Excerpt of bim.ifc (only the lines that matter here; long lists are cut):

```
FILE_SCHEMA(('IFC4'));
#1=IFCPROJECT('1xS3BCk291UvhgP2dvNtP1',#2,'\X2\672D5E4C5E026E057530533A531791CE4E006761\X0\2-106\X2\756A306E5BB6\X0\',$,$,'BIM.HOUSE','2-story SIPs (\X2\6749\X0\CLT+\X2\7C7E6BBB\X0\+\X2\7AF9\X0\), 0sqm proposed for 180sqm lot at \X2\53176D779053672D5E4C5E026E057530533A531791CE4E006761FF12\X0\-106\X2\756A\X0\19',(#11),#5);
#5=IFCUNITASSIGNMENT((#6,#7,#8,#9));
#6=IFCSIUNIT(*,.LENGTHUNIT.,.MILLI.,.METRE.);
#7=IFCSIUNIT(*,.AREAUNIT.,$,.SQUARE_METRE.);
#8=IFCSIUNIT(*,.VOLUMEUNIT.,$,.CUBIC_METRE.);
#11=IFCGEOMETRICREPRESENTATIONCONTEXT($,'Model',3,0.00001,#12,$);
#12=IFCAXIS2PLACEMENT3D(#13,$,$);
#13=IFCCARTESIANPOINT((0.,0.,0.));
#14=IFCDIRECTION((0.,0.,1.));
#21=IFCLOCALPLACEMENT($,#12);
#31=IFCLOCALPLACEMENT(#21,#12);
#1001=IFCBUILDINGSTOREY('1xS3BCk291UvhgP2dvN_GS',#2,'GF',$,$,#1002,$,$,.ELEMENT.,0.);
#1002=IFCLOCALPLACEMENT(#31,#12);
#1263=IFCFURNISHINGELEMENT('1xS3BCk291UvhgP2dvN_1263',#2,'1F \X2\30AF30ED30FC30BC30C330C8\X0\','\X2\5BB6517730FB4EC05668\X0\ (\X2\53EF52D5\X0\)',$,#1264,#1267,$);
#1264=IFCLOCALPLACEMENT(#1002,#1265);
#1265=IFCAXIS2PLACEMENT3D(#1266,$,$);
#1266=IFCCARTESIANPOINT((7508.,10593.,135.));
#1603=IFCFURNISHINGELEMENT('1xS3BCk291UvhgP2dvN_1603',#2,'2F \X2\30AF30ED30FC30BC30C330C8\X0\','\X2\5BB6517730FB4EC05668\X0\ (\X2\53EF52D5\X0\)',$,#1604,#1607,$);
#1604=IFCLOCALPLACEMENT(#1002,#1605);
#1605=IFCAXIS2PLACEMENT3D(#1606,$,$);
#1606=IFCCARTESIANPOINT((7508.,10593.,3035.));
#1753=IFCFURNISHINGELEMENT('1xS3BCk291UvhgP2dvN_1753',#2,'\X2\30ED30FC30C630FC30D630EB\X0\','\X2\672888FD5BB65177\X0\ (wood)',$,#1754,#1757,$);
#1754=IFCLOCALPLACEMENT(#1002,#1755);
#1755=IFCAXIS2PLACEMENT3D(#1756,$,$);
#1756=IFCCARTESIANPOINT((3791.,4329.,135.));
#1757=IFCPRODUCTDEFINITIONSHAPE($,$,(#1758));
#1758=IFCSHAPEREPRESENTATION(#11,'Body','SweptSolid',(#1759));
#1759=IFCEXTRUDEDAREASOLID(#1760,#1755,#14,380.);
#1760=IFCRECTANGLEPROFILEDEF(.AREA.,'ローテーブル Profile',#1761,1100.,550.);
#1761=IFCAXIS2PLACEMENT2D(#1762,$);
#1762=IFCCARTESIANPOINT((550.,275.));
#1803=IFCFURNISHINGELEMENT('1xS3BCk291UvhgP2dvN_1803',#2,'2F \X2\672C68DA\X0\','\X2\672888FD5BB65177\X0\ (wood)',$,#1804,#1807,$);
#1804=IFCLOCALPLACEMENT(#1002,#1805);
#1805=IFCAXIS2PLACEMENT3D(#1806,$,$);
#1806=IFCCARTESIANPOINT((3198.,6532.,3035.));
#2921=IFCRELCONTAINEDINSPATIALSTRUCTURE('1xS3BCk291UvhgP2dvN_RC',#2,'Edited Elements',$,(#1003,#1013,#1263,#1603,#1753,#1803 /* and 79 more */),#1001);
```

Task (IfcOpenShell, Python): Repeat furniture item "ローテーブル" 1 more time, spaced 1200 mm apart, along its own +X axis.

```python
import ifcopenshell
import ifcopenshell.api.geometry
import ifcopenshell.api.root
import ifcopenshell.util.element
import ifcopenshell.util.placement
import ifcopenshell.util.unit

model = ifcopenshell.open("bim.ifc")
unit_scale = ifcopenshell.util.unit.calculate_unit_scale(model)


def reuse_history(source, copy):
    """copy_class also copies each property set's owner history, people and application; keep the originals."""
    for rel in copy.IsDefinedBy:
        if rel.is_a("IfcRelDefinesByProperties") and (history := rel.RelatingPropertyDefinition.OwnerHistory):
            rel.RelatingPropertyDefinition.OwnerHistory = source.OwnerHistory
            ifcopenshell.util.element.remove_deep2(model, history)


source = model.by_id(1753)
base = ifcopenshell.util.placement.get_local_placement(source.ObjectPlacement)
step = base[:3, 0] * 1.2 / unit_scale

for i in range(1, 2):
    copy = ifcopenshell.api.root.copy_class(model, product=source)
    copy.Representation = ifcopenshell.util.element.copy_deep(
        model, source.Representation, exclude=["IfcGeometricRepresentationContext", "IfcRepresentationMap"]
    )
    reuse_history(source, copy)
    matrix = base.copy()
    matrix[:3, 3] += i * step
    print("added at", matrix[:3, 3].round(3) + 0.0)
    ifcopenshell.api.geometry.edit_object_placement(model, product=copy, matrix=matrix, is_si=False)

model.write("bim-out.ifc")
```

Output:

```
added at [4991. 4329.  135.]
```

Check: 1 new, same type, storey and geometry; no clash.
